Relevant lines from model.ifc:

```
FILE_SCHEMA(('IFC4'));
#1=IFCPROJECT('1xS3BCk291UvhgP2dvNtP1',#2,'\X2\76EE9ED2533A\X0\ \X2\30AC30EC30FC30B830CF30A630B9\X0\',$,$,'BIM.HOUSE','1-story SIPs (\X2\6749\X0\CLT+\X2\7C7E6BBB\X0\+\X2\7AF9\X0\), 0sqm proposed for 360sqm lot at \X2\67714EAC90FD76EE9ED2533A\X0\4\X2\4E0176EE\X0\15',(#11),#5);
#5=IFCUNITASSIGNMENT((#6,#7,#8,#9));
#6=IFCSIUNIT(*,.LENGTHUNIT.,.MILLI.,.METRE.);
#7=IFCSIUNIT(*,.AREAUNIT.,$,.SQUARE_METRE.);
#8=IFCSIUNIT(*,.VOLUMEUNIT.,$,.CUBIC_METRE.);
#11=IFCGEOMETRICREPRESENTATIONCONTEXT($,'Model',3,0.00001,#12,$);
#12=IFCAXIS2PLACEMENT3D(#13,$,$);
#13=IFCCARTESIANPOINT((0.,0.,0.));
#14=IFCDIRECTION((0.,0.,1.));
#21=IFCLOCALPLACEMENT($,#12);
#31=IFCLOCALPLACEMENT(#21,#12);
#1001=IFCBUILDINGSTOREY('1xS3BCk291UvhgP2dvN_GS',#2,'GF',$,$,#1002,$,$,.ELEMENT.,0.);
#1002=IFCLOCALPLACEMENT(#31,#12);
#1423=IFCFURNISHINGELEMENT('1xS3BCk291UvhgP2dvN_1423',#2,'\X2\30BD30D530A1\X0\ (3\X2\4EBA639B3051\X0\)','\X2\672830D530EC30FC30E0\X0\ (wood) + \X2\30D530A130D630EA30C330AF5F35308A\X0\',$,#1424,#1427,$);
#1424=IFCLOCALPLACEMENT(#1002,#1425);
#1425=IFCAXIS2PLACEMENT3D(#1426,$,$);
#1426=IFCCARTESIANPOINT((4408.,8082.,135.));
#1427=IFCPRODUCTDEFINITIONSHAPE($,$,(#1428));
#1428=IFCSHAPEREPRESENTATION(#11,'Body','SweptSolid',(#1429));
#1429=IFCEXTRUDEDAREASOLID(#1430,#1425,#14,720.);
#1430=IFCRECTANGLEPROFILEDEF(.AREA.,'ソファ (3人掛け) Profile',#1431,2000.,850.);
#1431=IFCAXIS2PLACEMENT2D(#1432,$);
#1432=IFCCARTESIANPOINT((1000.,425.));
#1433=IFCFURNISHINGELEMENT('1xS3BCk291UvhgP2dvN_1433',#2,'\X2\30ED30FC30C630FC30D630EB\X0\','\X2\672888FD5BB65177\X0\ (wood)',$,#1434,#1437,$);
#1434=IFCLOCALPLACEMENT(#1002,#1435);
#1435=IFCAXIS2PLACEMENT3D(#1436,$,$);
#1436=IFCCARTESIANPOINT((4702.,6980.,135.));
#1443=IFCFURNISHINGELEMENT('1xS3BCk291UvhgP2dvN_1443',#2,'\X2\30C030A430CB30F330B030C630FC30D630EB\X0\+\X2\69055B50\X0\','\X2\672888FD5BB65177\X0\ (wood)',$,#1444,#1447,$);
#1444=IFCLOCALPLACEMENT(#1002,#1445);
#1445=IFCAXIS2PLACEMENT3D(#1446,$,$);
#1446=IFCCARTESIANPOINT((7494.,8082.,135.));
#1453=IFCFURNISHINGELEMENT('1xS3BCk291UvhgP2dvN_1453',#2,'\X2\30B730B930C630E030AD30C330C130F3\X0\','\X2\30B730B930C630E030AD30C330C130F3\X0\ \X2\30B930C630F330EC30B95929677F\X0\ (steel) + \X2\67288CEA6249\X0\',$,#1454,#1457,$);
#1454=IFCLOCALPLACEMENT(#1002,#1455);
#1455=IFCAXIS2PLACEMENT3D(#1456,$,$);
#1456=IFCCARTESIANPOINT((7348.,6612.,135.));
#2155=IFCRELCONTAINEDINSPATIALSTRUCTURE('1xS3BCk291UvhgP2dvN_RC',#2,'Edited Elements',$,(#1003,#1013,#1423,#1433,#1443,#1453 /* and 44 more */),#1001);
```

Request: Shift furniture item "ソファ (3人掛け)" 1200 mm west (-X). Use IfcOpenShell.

```python
import ifcopenshell
import ifcopenshell.api.geometry
import ifcopenshell.util.placement
import ifcopenshell.util.unit

model = ifcopenshell.open("model.ifc")
unit_scale = ifcopenshell.util.unit.calculate_unit_scale(model)

item = model.by_guid("1xS3BCk291UvhgP2dvN_1423")
matrix = ifcopenshell.util.placement.get_local_placement(item.ObjectPlacement)
matrix[0, 3] -= 1.2 / unit_scale
ifcopenshell.api.geometry.edit_object_placement(model, product=item, matrix=matrix, is_si=False)

print(ifcopenshell.util.placement.get_local_placement(item.ObjectPlacement).round(3) + 0.0)

model.write("model_edited.ifc")
```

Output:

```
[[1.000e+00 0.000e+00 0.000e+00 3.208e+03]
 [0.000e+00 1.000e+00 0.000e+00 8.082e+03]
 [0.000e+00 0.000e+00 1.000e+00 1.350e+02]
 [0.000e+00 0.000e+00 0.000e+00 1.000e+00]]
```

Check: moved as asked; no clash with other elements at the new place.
